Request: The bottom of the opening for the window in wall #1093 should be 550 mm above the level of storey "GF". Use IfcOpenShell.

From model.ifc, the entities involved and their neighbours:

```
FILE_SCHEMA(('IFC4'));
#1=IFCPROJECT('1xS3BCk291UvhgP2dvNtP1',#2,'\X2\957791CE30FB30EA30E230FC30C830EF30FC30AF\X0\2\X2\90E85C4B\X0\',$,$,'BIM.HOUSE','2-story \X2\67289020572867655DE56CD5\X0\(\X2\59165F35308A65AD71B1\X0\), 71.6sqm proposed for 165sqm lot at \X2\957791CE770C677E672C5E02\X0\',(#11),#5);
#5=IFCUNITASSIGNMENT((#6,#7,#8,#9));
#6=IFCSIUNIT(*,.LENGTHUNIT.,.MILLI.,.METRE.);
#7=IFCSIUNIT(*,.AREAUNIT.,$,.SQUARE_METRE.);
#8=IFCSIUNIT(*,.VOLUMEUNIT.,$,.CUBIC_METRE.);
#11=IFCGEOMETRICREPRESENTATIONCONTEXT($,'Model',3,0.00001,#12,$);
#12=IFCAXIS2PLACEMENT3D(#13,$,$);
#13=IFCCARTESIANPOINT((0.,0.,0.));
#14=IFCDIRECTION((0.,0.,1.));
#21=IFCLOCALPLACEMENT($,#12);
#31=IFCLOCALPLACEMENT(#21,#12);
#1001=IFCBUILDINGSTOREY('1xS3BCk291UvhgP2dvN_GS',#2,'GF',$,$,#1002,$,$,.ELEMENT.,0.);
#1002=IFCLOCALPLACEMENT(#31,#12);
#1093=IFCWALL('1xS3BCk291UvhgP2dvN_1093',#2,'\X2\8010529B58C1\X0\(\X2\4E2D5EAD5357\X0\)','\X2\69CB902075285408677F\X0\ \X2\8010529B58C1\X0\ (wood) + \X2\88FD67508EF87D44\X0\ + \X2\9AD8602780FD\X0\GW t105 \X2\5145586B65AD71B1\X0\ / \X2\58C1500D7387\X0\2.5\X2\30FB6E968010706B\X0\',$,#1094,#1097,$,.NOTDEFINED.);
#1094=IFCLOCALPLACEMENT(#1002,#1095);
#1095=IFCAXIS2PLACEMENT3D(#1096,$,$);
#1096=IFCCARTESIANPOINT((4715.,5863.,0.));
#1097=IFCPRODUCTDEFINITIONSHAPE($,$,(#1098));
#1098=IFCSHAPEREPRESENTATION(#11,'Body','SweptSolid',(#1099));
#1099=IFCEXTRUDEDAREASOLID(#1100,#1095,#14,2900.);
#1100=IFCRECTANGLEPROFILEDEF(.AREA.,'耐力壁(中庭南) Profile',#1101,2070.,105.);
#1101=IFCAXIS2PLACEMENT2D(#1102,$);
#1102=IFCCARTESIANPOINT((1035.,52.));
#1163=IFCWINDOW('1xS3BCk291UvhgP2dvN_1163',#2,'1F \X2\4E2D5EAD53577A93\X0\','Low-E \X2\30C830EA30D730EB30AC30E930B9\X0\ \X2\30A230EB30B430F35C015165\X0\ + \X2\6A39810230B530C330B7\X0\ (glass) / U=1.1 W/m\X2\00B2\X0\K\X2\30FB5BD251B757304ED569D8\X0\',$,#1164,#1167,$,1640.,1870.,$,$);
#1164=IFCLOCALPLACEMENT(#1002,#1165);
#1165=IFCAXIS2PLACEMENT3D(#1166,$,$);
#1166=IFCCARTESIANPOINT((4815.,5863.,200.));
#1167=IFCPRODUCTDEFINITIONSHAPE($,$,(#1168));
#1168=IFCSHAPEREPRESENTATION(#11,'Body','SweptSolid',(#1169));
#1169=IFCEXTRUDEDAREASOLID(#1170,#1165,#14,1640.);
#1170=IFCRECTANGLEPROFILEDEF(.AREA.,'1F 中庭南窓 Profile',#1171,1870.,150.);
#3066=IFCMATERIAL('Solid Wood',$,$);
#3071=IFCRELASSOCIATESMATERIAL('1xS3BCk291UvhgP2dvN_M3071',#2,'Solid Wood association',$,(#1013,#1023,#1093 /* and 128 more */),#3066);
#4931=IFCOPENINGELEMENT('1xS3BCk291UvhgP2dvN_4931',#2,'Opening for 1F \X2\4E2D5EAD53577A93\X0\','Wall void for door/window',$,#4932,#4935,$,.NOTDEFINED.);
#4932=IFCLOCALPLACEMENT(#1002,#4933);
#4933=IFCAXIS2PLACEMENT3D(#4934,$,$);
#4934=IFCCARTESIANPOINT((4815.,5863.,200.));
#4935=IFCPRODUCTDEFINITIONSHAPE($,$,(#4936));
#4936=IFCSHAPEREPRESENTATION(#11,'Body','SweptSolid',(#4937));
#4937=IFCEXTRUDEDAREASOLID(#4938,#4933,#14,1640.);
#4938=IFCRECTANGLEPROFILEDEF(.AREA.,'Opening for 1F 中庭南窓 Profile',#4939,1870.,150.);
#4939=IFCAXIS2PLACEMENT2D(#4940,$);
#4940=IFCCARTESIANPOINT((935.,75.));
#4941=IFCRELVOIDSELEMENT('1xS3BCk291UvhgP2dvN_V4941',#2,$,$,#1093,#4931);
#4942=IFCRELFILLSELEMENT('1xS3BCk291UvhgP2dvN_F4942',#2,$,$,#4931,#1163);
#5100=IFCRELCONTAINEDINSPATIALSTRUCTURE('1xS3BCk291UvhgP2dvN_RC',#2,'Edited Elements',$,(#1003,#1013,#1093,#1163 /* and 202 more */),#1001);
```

```python
import numpy as np
import ifcopenshell
import ifcopenshell.api.geometry
import ifcopenshell.geom
import ifcopenshell.util.element
import ifcopenshell.util.placement
import ifcopenshell.util.shape
import ifcopenshell.util.unit

model = ifcopenshell.open("model.ifc")
unit_scale = ifcopenshell.util.unit.calculate_unit_scale(model)

window = model.by_id(1163)
opening = window.FillsVoids[0].RelatingOpeningElement
storey = ifcopenshell.util.element.get_container(window, ifc_class="IfcBuildingStorey")
level = ifcopenshell.util.placement.get_local_placement(storey.ObjectPlacement)[2, 3]

# The opening's origin need not be at the sill, so measure its lowest point.
shape = ifcopenshell.geom.create_shape(ifcopenshell.geom.settings(), opening)
bottom = ifcopenshell.util.shape.get_shape_bottom_elevation(shape, shape.geometry) / unit_scale
dz = level + 0.55 / unit_scale - bottom

shift = np.array([0.0, 0.0, dz])
# The window is not placed relative to its opening, so move both.
for product in (opening, window):
    matrix = ifcopenshell.util.placement.get_local_placement(product.ObjectPlacement)
    matrix[:3, 3] += shift
    ifcopenshell.api.geometry.edit_object_placement(model, product=product, matrix=matrix, is_si=False)

print(f"moved by {dz * unit_scale:+.3f} m")

model.write("model_rev.ifc")
```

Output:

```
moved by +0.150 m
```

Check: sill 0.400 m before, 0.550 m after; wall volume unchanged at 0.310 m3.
